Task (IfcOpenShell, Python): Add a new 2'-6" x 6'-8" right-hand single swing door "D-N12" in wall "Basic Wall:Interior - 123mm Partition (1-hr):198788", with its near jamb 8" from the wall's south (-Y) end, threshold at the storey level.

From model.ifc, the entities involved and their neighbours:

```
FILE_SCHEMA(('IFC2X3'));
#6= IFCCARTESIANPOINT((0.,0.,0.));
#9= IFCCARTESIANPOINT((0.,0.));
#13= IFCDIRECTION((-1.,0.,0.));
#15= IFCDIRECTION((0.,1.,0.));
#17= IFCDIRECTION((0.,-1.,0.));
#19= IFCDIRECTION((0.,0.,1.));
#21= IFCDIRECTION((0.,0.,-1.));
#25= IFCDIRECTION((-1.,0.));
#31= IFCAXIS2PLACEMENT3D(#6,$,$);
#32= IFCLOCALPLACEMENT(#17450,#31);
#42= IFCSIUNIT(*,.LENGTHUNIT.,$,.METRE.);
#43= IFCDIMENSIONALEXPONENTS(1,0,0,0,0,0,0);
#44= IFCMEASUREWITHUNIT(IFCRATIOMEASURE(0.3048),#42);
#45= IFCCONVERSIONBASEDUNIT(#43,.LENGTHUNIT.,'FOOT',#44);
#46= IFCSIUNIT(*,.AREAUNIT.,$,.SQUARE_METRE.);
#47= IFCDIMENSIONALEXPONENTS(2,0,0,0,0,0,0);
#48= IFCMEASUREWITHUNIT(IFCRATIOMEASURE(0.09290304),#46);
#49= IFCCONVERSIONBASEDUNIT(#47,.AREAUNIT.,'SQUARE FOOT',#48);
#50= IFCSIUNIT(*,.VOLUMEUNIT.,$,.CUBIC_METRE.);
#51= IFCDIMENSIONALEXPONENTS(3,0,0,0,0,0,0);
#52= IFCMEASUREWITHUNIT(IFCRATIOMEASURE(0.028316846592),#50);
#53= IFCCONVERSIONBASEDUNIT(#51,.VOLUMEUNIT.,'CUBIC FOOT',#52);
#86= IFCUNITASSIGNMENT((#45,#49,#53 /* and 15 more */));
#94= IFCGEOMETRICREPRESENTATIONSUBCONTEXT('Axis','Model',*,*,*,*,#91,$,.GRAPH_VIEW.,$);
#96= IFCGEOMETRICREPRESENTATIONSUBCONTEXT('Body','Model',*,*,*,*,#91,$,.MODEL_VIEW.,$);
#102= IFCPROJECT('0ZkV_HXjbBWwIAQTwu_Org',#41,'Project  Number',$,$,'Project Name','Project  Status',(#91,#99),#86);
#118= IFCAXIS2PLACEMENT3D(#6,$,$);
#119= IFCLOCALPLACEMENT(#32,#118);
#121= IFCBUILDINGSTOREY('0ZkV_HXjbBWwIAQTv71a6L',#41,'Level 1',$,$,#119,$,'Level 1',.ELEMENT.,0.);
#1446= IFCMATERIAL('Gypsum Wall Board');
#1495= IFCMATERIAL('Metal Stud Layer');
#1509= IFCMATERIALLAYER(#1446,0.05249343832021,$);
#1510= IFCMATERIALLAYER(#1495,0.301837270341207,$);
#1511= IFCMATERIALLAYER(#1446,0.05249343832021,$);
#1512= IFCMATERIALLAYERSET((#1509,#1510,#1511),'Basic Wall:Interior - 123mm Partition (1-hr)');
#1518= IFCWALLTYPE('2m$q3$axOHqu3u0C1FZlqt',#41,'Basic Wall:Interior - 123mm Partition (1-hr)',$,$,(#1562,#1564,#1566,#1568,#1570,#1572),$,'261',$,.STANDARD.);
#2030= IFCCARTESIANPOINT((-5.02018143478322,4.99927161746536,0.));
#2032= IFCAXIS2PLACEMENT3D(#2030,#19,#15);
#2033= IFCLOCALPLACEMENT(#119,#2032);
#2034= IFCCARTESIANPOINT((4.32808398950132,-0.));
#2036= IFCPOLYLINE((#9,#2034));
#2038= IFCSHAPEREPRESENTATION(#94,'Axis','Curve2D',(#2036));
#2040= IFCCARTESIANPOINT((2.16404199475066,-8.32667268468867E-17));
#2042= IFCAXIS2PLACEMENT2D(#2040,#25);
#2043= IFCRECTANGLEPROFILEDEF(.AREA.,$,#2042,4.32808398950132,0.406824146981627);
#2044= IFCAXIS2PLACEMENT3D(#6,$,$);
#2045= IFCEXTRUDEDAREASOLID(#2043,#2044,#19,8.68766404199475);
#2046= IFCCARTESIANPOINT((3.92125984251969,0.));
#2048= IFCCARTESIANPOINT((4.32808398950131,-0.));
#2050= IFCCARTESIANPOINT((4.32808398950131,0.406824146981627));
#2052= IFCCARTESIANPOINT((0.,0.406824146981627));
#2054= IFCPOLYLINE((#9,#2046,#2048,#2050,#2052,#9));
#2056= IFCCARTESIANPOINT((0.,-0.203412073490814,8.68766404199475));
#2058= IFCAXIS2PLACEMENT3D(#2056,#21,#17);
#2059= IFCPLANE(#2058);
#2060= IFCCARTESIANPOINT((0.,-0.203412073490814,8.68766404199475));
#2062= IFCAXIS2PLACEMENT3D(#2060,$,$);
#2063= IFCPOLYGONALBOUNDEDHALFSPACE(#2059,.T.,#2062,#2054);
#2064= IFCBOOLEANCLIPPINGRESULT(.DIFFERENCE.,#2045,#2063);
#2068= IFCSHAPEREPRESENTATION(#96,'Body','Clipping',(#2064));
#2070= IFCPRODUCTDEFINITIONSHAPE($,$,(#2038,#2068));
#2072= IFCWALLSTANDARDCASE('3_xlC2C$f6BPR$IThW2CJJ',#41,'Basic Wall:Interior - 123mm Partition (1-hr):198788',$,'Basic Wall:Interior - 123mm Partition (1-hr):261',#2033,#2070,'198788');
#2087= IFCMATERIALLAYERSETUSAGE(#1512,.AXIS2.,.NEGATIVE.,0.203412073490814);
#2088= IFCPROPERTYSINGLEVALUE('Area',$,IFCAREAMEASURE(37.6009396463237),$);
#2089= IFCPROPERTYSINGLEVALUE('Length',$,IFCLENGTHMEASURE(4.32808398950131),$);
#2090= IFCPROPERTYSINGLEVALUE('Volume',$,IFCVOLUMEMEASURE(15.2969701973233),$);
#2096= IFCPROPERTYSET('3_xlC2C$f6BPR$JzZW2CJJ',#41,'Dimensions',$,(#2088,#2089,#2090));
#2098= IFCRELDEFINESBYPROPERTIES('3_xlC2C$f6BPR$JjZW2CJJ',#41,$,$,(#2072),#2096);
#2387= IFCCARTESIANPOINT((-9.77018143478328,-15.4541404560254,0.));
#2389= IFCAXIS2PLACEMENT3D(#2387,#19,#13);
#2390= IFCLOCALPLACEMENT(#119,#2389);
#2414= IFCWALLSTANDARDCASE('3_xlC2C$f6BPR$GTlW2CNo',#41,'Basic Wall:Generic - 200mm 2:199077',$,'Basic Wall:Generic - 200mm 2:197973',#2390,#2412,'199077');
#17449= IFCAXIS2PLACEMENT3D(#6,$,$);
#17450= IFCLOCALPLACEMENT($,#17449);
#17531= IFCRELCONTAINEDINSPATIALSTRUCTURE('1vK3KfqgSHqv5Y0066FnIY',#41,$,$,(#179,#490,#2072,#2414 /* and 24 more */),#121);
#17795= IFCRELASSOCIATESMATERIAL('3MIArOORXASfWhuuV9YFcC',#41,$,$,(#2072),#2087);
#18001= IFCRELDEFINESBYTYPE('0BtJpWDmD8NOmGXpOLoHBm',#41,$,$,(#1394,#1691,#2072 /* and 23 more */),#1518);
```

```python
import numpy as np
import ifcopenshell
import ifcopenshell.api.feature
import ifcopenshell.api.geometry
import ifcopenshell.api.pset
import ifcopenshell.api.root
import ifcopenshell.api.spatial
import ifcopenshell.api.type
import ifcopenshell.geom
import ifcopenshell.util.element
import ifcopenshell.util.placement
import ifcopenshell.util.representation
import ifcopenshell.util.shape
import ifcopenshell.util.unit

model = ifcopenshell.open("model.ifc")
unit_scale = ifcopenshell.util.unit.calculate_unit_scale(model)
area_scale = ifcopenshell.util.unit.calculate_unit_scale(model, "AREAUNIT")
volume_scale = ifcopenshell.util.unit.calculate_unit_scale(model, "VOLUMEUNIT")
settings = ifcopenshell.geom.settings()


def volume(element):
    """Net volume in cubic metres, openings subtracted."""
    shape = ifcopenshell.geom.create_shape(settings, element)
    return ifcopenshell.util.shape.get_volume(shape.geometry)


wall = model.by_guid("3_xlC2C$f6BPR$IThW2CJJ")
storey = ifcopenshell.util.element.get_container(wall, ifc_class="IfcBuildingStorey")
context = ifcopenshell.util.representation.get_context(model, "Model", "Body", "MODEL_VIEW")
before = volume(wall)

width, height, from_end, sill = 0.762, 2.032, 0.2032, 0.0  # metres

# The wall runs along its own X axis, and the end named is its -X end.
wall_shape = ifcopenshell.geom.create_shape(settings, wall)
x, y, z = ifcopenshell.util.shape.get_vertices(wall_shape.geometry).T
start = x.min() + from_end
face, thickness = float(y.min()), float(y.max() - y.min())
wall_matrix = ifcopenshell.util.placement.get_local_placement(wall.ObjectPlacement)
level = ifcopenshell.util.placement.get_local_placement(storey.ObjectPlacement)[2, 3]


def in_wall(x, y):
    """Placement at x, y metres in the wall's axes, at sill height."""
    matrix = wall_matrix.copy()
    matrix[:, 3] = wall_matrix @ np.array([x / unit_scale, y / unit_scale, 0.0, 1.0])
    matrix[2, 3] = level + sill / unit_scale
    return matrix


# Opening: a box that overshoots both wall faces by 50 mm.
opening = ifcopenshell.api.root.create_entity(model, ifc_class="IfcOpeningElement")
box = ifcopenshell.api.geometry.add_wall_representation(
    model, context=context, length=width, height=height, thickness=thickness + 0.1
)
ifcopenshell.api.geometry.assign_representation(model, product=opening, representation=box)
ifcopenshell.api.geometry.edit_object_placement(model, product=opening, matrix=in_wall(start, face - 0.05), is_si=False)
ifcopenshell.api.feature.add_feature(model, feature=opening, element=wall)

door = ifcopenshell.api.root.create_entity(model, ifc_class="IfcDoor", name="D-N12")
door.OverallWidth, door.OverallHeight = width / unit_scale, height / unit_scale
body = ifcopenshell.api.geometry.add_door_representation(
    model,
    context=context,
    overall_width=door.OverallWidth,
    overall_height=door.OverallHeight,
    operation_type="SINGLE_SWING_RIGHT",
    lining_properties={"LiningDepth": thickness / unit_scale, "ThresholdDepth": thickness / unit_scale},
)
ifcopenshell.api.geometry.assign_representation(model, product=door, representation=body)
ifcopenshell.api.spatial.assign_container(model, products=[door], relating_structure=storey)
fills = ifcopenshell.api.feature.add_filling(model, opening=opening, element=door)
fills.OwnerHistory = door.OwnerHistory  # required in IFC2X3

# IFC2X3 keeps the operation on the door style.
style = ifcopenshell.api.root.create_entity(model, ifc_class="IfcDoorStyle", name="D-N12")
style.OperationType, style.ConstructionType = "SINGLE_SWING_RIGHT", "NOTDEFINED"
style.ParameterTakesPrecedence = style.Sizeable = False
ifcopenshell.api.type.assign_type(model, related_objects=[door], relating_type=style)

# The lining spans the wall, so the door starts at the wall face.
ifcopenshell.api.geometry.edit_object_placement(model, product=door, matrix=in_wall(start, face), is_si=False)

after = volume(wall)

# Update the wall's stored quantities.
pset = model.by_id(ifcopenshell.util.element.get_pset(wall, "Dimensions", should_inherit=False)["id"])
ifcopenshell.api.pset.edit_pset(model, pset=pset, properties={
    "Area": model.create_entity("IfcAreaMeasure", after / thickness / area_scale),
    "Volume": model.create_entity("IfcVolumeMeasure", after / volume_scale),
})

print(f"wall volume {before:.3f} -> {after:.3f} m3")

model.write("model_v2.ifc")
```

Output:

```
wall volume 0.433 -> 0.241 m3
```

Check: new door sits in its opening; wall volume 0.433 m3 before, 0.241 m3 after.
